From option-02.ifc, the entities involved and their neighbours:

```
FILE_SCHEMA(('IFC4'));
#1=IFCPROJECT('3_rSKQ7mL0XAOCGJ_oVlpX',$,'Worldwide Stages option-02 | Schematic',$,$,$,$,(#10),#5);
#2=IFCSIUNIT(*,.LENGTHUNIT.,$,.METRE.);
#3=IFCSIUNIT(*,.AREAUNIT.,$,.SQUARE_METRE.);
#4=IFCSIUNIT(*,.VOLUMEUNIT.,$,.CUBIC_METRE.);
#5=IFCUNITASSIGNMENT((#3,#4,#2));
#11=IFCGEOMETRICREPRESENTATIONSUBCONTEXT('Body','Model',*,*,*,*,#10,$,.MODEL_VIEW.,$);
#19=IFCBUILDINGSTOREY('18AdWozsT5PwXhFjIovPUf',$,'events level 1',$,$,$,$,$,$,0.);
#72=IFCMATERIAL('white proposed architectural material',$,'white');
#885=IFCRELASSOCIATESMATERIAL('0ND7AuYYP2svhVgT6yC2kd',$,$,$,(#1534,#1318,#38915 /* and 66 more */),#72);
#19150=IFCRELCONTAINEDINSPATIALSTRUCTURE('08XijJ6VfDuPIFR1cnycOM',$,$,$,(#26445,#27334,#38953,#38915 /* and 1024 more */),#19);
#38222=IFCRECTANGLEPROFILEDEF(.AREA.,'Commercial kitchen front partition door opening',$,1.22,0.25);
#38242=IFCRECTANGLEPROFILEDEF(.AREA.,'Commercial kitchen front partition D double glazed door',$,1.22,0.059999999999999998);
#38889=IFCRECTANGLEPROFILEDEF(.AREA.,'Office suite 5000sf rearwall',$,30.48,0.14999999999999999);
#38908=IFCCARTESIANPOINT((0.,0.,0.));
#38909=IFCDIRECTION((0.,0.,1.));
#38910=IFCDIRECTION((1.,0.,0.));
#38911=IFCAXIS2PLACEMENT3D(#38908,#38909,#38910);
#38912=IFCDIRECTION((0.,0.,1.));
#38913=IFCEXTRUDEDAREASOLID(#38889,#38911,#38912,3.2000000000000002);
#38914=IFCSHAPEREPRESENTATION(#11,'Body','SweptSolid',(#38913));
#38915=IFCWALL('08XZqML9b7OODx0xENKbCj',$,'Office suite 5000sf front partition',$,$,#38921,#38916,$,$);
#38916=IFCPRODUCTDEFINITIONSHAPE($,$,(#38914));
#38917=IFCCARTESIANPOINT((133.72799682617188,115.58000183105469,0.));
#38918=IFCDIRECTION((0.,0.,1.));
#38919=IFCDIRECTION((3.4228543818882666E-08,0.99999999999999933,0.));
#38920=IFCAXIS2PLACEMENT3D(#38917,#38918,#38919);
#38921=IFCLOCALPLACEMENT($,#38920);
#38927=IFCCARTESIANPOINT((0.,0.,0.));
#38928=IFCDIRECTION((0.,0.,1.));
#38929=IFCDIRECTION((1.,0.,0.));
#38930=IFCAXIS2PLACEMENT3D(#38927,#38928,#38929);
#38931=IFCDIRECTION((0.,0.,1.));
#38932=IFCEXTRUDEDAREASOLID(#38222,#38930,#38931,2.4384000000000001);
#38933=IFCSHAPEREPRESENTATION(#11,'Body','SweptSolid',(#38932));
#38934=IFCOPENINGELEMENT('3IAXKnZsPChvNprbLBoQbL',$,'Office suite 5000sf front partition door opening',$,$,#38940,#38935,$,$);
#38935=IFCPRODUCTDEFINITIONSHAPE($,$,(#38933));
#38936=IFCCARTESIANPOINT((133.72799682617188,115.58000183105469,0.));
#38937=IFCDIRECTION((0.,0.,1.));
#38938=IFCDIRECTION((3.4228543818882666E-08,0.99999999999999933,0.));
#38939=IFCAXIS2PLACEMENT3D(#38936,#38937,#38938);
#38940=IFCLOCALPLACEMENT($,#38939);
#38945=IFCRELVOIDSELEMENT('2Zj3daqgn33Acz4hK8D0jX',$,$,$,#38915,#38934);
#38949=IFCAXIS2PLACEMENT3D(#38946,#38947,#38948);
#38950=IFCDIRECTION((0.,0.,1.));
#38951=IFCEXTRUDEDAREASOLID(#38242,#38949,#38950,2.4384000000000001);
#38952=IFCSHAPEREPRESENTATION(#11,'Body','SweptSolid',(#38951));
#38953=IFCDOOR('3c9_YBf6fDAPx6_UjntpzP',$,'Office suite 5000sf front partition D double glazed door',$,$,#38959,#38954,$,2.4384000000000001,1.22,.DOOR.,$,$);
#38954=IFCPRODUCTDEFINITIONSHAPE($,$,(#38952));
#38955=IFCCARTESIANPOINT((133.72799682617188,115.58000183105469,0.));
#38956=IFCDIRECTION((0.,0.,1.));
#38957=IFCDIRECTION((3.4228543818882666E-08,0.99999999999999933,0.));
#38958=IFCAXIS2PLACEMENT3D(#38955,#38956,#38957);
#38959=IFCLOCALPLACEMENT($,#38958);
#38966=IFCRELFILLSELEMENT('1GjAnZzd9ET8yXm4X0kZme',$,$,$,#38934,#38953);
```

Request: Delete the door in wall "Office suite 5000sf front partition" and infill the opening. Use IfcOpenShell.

```python
import ifcopenshell
import ifcopenshell.api.feature
import ifcopenshell.api.root
import ifcopenshell.geom
import ifcopenshell.util.shape

model = ifcopenshell.open("option-02.ifc")
settings = ifcopenshell.geom.settings()


def volume(element):
    """Net volume in cubic metres, openings subtracted."""
    shape = ifcopenshell.geom.create_shape(settings, element)
    return ifcopenshell.util.shape.get_volume(shape.geometry)


door = model.by_guid("3c9_YBf6fDAPx6_UjntpzP")
opening = door.FillsVoids[0].RelatingOpeningElement
wall = opening.VoidsElements[0].RelatingBuildingElement
before = volume(wall)

ifcopenshell.api.root.remove_product(model, product=door)
ifcopenshell.api.feature.remove_feature(model, feature=opening)

after = volume(wall)

print(f"wall volume {before:.3f} -> {after:.3f} m3")

model.write("option-02_rev.ifc")
```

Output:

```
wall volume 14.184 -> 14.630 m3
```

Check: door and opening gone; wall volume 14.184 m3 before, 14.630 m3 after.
